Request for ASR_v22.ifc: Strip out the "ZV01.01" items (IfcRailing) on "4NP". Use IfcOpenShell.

First a look at what the model holds.

```python
import ifcopenshell
import ifcopenshell.util.element

model = ifcopenshell.open("ASR_v22.ifc")
print(model.schema)
storey = next(s for s in model.by_type("IfcBuildingStorey") if s.Name == "4NP")
railings = [e for e in ifcopenshell.util.element.get_decomposition(storey) if e.is_a("IfcRailing")]
seen = {}
for e in railings:
    element_type = ifcopenshell.util.element.get_type(e)
    name = element_type.Name if element_type not in (None, e) else None
    seen[name] = seen.get(name, 0) + 1
for name, count in sorted(seen.items(), key=str):
    print(count, "x", name)
```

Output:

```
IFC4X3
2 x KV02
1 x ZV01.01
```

```python
import ifcopenshell
import ifcopenshell.api.root
import ifcopenshell.util.element

model = ifcopenshell.open("ASR_v22.ifc")

storey = next(s for s in model.by_type("IfcBuildingStorey") if s.Name == "4NP")
railings = [e for e in ifcopenshell.util.element.get_decomposition(storey) if e.is_a("IfcRailing")]
targets = [e for e in railings if (t := ifcopenshell.util.element.get_type(e)) not in (None, e) and t.Name == "ZV01.01"]

for e in targets:
    ifcopenshell.api.root.remove_product(model, product=e)
print(len(targets), "removed")

model.write("ASR_v22_v2.ifc")
```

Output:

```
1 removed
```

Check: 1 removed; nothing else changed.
